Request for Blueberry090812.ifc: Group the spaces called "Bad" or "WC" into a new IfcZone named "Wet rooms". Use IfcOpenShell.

First a look at what the model holds.

```python
import ifcopenshell

model = ifcopenshell.open("Blueberry090812.ifc")
print(model.schema)
seen = {}
for space in model.by_type("IfcSpace"):
    seen[space.LongName] = seen.get(space.LongName, 0) + 1
for name, count in sorted(seen.items(), key=str):
    print(count, "x", name)
print("zones:", [z.Name for z in model.by_type("IfcZone")][:20])
```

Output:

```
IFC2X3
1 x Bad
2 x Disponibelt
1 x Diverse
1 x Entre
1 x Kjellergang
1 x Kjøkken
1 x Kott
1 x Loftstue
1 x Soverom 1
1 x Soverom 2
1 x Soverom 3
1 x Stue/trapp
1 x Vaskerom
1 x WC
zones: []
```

```python
import ifcopenshell
import ifcopenshell.api.group
import ifcopenshell.api.root

model = ifcopenshell.open("Blueberry090812.ifc")

names = {"Bad", "WC"}
spaces = [s for s in model.by_type("IfcSpace") if s.LongName in names]

zone = ifcopenshell.api.root.create_entity(model, ifc_class="IfcZone", name="Wet rooms")
ifcopenshell.api.group.assign_group(model, products=spaces, group=zone)
print(len(spaces), "spaces in", zone.Name)

model.write("Blueberry090812_v2.ifc")
```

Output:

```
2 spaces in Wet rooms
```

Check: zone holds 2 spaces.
